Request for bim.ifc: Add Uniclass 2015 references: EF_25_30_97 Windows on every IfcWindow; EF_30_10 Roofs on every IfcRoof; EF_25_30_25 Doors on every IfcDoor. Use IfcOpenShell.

First a look at what the model holds.

```python
import ifcopenshell

model = ifcopenshell.open("bim.ifc")
print(model.schema)
print("classifications:", [c.Name for c in model.by_type("IfcClassification")])
for ifc_class in ("IfcDoor", "IfcRoof", "IfcStair", "IfcWall", "IfcWindow"):
    print(ifc_class, len(model.by_type(ifc_class)))
```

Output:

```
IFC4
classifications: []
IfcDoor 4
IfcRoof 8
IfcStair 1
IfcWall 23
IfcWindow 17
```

```python
import ifcopenshell
import ifcopenshell.api.classification

model = ifcopenshell.open("bim.ifc")

system = ifcopenshell.api.classification.add_classification(model, classification="Uniclass 2015")

codes = {
    "IfcWindow": ("EF_25_30_97", "Windows"),
    "IfcRoof": ("EF_30_10", "Roofs"),
    "IfcDoor": ("EF_25_30_25", "Doors"),
}
for ifc_class, (code, name) in codes.items():
    products = model.by_type(ifc_class)
    ifcopenshell.api.classification.add_reference(
        model, products=products, classification=system, identification=code, name=name
    )
    print(code, len(products))

model.write("bim_v2.ifc")
```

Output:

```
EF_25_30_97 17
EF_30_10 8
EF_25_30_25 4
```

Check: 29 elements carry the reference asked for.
